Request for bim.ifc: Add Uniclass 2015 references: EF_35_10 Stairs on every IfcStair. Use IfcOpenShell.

First a look at what the model holds.

```python
import ifcopenshell

model = ifcopenshell.open("bim.ifc")
print(model.schema)
print("classifications:", [c.Name for c in model.by_type("IfcClassification")])
for ifc_class in ("IfcDoor", "IfcRoof", "IfcStair", "IfcWall", "IfcWindow"):
    print(ifc_class, len(model.by_type(ifc_class)))
```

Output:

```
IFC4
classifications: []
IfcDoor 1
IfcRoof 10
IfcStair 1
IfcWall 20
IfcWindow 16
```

```python
import ifcopenshell
import ifcopenshell.api.classification

model = ifcopenshell.open("bim.ifc")

system = ifcopenshell.api.classification.add_classification(model, classification="Uniclass 2015")

codes = {
    "IfcStair": ("EF_35_10", "Stairs"),
}
for ifc_class, (code, name) in codes.items():
    products = model.by_type(ifc_class)
    ifcopenshell.api.classification.add_reference(
        model, products=products, classification=system, identification=code, name=name
    )
    print(code, len(products))

model.write("bim-out.ifc")
```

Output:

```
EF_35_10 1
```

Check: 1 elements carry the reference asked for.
